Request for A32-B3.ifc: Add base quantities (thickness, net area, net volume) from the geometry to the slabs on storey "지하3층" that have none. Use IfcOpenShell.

First a look at what the model holds.

```python
import ifcopenshell
import ifcopenshell.util.element
import ifcopenshell.util.unit

model = ifcopenshell.open("A32-B3.ifc")
print(model.schema)
for unit_type in ("LENGTHUNIT", "AREAUNIT", "VOLUMEUNIT"):
    print(unit_type, ifcopenshell.util.unit.calculate_unit_scale(model, unit_type))
storey = next(s for s in model.by_type("IfcBuildingStorey") if s.Name == "지하3층")
slabs = [e for e in ifcopenshell.util.element.get_decomposition(storey) if e.is_a("IfcSlab")]
for e in sorted(slabs, key=lambda e: e.id()):
    print(e.id(), e.is_a(), e.Name, list(ifcopenshell.util.element.get_psets(e, qtos_only=True)), sep=" | ")
```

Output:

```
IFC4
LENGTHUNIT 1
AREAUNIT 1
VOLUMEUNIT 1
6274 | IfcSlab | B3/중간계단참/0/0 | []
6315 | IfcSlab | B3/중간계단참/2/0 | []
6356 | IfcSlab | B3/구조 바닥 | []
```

```python
import ifcopenshell
import ifcopenshell.api.pset
import ifcopenshell.geom
import ifcopenshell.util.element
import ifcopenshell.util.shape
import ifcopenshell.util.unit

model = ifcopenshell.open("A32-B3.ifc")
unit_scale = ifcopenshell.util.unit.calculate_unit_scale(model)
area_scale = ifcopenshell.util.unit.calculate_unit_scale(model, "AREAUNIT")
volume_scale = ifcopenshell.util.unit.calculate_unit_scale(model, "VOLUMEUNIT")
settings = ifcopenshell.geom.settings()

storey = next(s for s in model.by_type("IfcBuildingStorey") if s.Name == "지하3층")
slabs = [e for e in ifcopenshell.util.element.get_decomposition(storey) if e.is_a("IfcSlab")]

for e in sorted(slabs, key=lambda e: e.id()):
    if ifcopenshell.util.element.get_psets(e, qtos_only=True, should_inherit=False):
        continue
    # Geometry comes back in metres, in the element's own axes.
    shape = ifcopenshell.geom.create_shape(settings, e)
    values = {
        "Width": ifcopenshell.util.shape.get_z(shape.geometry) / unit_scale,
        "NetArea": ifcopenshell.util.shape.get_footprint_area(shape.geometry) / area_scale,
        "NetVolume": ifcopenshell.util.shape.get_volume(shape.geometry) / volume_scale,
    }
    qto = ifcopenshell.api.pset.add_qto(model, product=e, name="Qto_SlabBaseQuantities")
    ifcopenshell.api.pset.edit_qto(model, qto=qto, properties=values)
    print(e.id(), {k: round(v, 3) for k, v in values.items()})

model.write("A32-B3_updated.ifc")
```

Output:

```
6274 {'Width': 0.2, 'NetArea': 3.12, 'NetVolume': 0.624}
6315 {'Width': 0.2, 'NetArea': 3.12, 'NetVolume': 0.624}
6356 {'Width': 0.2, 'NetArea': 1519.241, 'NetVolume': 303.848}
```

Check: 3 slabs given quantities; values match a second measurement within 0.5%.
